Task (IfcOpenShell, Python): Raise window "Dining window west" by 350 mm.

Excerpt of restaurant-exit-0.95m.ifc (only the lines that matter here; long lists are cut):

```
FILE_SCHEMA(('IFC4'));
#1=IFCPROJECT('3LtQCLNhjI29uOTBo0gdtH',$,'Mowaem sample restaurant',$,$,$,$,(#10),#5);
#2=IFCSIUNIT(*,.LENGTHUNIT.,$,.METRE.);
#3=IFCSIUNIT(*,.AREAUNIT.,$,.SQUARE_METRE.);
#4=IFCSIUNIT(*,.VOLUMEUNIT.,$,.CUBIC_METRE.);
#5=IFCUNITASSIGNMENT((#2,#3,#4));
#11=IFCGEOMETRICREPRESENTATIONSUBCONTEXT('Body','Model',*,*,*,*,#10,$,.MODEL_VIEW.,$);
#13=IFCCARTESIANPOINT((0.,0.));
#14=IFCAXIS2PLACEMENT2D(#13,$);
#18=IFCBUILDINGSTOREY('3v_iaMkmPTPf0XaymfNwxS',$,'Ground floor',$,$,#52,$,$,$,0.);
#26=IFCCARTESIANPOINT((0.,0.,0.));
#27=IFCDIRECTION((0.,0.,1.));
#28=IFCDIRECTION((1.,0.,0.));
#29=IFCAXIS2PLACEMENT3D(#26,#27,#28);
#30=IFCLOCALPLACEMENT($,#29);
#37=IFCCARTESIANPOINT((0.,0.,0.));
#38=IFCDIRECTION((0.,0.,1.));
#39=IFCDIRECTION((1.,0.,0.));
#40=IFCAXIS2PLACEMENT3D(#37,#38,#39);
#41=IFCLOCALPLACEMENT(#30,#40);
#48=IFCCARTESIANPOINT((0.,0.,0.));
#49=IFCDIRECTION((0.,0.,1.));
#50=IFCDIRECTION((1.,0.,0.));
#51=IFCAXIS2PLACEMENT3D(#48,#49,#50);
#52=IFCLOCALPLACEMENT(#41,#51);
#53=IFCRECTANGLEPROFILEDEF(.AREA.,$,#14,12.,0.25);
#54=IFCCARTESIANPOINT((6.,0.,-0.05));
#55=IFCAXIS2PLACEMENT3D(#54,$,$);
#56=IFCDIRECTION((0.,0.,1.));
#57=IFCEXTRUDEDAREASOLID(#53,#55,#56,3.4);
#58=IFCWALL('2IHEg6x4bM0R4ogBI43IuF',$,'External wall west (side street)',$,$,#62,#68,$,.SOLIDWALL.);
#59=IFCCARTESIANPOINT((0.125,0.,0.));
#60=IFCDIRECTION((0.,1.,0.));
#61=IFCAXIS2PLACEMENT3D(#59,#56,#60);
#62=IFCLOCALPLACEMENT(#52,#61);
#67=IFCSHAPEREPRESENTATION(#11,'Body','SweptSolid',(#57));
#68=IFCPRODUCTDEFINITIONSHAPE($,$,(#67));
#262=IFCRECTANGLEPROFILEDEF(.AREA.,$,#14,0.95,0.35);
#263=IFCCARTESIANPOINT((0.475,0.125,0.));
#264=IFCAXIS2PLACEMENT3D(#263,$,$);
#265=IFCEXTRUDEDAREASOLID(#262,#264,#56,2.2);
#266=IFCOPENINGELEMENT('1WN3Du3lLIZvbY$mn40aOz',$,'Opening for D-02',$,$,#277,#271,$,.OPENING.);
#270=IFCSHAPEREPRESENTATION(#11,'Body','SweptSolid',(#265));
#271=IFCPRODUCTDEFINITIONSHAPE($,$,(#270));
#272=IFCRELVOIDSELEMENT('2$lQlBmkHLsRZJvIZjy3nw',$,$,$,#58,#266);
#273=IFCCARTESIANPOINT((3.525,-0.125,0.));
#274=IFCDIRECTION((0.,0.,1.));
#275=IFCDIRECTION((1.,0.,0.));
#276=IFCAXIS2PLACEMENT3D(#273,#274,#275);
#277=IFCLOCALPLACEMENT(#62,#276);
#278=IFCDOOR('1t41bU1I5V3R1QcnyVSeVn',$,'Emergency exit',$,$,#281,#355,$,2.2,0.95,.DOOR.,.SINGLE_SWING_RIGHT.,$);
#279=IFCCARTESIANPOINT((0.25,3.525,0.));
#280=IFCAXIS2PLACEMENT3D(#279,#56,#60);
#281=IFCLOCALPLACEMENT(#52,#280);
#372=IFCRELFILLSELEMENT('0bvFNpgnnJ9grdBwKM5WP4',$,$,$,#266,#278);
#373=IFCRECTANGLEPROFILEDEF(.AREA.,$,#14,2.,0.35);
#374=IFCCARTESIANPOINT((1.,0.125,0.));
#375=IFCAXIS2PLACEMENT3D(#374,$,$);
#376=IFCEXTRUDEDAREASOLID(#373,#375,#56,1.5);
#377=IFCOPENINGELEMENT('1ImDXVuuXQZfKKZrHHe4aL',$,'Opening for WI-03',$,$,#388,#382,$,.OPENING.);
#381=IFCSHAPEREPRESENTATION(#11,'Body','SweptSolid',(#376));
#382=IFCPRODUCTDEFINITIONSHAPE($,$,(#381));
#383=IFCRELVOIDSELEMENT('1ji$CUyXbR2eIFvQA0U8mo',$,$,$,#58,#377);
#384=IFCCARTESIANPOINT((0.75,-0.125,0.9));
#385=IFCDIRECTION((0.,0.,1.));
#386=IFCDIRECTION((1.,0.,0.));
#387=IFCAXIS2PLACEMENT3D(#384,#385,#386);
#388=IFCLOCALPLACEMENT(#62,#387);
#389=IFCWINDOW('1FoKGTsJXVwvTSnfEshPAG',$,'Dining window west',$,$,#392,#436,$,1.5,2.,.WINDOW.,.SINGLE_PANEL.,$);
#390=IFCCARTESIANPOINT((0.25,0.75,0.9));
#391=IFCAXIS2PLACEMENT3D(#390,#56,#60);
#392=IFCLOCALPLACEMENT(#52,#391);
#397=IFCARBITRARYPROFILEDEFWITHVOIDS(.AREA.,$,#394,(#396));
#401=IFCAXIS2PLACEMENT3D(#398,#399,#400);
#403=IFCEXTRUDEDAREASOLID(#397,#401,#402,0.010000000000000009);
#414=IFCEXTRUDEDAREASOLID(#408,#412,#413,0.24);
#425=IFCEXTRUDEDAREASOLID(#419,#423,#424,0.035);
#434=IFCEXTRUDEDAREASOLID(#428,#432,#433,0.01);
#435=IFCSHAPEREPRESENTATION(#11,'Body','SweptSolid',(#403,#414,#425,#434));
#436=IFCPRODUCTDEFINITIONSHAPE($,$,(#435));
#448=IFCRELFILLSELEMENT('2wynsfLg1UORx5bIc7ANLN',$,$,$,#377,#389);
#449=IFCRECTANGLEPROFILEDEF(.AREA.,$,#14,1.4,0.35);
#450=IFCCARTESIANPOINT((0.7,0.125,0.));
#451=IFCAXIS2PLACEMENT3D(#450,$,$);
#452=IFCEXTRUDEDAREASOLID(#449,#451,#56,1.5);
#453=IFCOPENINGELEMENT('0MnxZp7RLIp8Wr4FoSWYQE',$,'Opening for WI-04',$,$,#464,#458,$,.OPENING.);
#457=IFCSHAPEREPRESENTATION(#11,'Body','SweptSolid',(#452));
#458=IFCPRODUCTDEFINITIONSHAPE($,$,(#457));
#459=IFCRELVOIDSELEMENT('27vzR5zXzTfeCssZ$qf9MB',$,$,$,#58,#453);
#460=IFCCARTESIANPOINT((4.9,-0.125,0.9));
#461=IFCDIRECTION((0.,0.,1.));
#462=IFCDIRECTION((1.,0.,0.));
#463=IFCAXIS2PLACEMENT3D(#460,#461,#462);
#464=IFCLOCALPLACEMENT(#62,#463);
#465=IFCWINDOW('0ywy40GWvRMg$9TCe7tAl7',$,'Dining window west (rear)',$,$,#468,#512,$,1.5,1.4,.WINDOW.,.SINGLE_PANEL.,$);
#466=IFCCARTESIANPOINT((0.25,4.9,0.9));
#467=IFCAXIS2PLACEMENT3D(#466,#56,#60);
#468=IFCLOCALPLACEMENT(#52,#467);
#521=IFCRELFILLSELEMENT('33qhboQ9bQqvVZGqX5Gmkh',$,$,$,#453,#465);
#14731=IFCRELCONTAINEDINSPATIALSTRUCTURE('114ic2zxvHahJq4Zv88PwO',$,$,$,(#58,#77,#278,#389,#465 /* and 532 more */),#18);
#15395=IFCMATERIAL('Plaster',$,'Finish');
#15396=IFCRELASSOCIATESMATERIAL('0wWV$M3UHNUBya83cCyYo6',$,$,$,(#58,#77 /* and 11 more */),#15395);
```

```python
import numpy as np
import ifcopenshell
import ifcopenshell.api.geometry
import ifcopenshell.util.placement
import ifcopenshell.util.unit

model = ifcopenshell.open("restaurant-exit-0.95m.ifc")
unit_scale = ifcopenshell.util.unit.calculate_unit_scale(model)

window = model.by_guid("1FoKGTsJXVwvTSnfEshPAG")
opening = window.FillsVoids[0].RelatingOpeningElement
dz = 0.35 / unit_scale

shift = np.array([0.0, 0.0, dz])
# The window is not placed relative to its opening, so move both.
for product in (opening, window):
    matrix = ifcopenshell.util.placement.get_local_placement(product.ObjectPlacement)
    matrix[:3, 3] += shift
    ifcopenshell.api.geometry.edit_object_placement(model, product=product, matrix=matrix, is_si=False)

print(f"moved by {dz * unit_scale:+.3f} m")

model.write("restaurant-exit-0.95m_rev.ifc")
```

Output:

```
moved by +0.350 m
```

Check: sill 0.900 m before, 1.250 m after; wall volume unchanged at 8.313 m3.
